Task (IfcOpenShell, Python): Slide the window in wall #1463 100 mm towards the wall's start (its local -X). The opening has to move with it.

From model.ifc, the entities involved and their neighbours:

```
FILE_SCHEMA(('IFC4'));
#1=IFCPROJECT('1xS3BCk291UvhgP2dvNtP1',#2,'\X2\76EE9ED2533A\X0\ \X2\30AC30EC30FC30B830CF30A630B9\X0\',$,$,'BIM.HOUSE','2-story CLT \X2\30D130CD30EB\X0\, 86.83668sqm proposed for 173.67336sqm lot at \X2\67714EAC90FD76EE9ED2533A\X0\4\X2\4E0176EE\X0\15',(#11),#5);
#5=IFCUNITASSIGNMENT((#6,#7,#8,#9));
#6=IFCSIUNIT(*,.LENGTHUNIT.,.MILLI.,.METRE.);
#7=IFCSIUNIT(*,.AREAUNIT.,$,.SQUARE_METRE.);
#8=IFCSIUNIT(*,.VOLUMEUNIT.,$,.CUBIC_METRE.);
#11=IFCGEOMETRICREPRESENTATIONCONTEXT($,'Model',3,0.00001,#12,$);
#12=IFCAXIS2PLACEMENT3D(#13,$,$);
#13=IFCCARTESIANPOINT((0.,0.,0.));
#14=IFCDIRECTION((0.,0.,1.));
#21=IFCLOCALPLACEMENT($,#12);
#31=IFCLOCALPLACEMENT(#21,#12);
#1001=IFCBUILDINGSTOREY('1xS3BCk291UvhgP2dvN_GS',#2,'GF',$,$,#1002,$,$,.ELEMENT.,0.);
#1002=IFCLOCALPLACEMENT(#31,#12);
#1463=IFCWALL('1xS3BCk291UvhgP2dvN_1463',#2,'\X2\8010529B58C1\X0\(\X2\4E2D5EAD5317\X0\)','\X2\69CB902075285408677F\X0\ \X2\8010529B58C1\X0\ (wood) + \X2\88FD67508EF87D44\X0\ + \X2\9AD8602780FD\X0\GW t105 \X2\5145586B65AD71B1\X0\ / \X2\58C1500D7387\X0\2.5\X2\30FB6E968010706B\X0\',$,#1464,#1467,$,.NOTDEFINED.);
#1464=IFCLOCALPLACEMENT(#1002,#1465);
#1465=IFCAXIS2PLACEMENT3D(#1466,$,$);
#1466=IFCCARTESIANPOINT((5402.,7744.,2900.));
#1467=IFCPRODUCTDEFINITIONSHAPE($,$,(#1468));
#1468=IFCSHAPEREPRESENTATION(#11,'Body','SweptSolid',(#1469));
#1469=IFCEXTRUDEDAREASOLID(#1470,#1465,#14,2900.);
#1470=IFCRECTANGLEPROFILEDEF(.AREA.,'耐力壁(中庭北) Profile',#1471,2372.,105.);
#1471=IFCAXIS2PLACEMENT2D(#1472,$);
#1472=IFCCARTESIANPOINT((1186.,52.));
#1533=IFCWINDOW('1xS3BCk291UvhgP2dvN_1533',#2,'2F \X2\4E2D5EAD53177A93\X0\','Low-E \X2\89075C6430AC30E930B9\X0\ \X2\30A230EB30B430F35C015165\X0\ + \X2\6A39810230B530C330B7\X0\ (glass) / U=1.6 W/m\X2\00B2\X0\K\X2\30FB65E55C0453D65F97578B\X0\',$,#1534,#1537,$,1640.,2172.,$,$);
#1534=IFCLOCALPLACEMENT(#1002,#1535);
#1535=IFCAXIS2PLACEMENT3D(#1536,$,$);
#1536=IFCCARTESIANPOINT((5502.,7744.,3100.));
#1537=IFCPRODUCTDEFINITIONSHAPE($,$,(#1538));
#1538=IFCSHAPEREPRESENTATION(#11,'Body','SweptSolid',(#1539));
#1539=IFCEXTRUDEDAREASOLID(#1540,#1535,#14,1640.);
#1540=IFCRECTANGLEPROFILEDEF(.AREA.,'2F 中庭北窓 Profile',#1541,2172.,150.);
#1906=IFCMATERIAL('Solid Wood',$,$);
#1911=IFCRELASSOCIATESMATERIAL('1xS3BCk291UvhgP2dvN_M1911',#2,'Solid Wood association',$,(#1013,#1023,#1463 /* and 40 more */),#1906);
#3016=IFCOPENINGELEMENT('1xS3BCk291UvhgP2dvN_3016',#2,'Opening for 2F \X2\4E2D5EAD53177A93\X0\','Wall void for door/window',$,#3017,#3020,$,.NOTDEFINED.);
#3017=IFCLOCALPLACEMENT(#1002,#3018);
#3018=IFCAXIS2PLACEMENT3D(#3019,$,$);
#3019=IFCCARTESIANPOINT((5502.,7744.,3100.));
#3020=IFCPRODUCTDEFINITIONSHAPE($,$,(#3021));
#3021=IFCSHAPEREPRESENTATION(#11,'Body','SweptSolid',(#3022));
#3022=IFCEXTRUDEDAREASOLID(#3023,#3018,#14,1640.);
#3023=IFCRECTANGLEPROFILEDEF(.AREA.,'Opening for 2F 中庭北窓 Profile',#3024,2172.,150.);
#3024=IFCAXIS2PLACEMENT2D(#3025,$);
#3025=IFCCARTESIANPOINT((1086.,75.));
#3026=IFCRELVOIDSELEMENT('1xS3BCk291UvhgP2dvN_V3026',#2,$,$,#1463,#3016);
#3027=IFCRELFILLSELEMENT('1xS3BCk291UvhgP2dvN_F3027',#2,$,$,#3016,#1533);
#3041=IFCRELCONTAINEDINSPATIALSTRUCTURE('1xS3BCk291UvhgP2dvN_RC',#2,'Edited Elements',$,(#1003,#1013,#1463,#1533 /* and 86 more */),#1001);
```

```python
import ifcopenshell
import ifcopenshell.api.geometry
import ifcopenshell.util.placement
import ifcopenshell.util.unit

model = ifcopenshell.open("model.ifc")
unit_scale = ifcopenshell.util.unit.calculate_unit_scale(model)

window = model.by_guid("1xS3BCk291UvhgP2dvN_1533")
opening = window.FillsVoids[0].RelatingOpeningElement
wall = opening.VoidsElements[0].RelatingBuildingElement

wall_matrix = ifcopenshell.util.placement.get_local_placement(wall.ObjectPlacement)
shift = wall_matrix[:3, 0] * -0.1 / unit_scale
before = ifcopenshell.util.placement.get_local_placement(window.ObjectPlacement)[:3, 3].copy()

# The window is not placed relative to its opening, so move both.
for product in (opening, window):
    matrix = ifcopenshell.util.placement.get_local_placement(product.ObjectPlacement)
    matrix[:3, 3] += shift
    ifcopenshell.api.geometry.edit_object_placement(model, product=product, matrix=matrix, is_si=False)

after = ifcopenshell.util.placement.get_local_placement(window.ObjectPlacement)[:3, 3]
print("window moved by", (after - before).round(3) + 0.0)

model.write("model_rev.ifc")
```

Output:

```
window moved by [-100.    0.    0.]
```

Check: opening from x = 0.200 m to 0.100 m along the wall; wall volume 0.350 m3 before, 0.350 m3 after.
